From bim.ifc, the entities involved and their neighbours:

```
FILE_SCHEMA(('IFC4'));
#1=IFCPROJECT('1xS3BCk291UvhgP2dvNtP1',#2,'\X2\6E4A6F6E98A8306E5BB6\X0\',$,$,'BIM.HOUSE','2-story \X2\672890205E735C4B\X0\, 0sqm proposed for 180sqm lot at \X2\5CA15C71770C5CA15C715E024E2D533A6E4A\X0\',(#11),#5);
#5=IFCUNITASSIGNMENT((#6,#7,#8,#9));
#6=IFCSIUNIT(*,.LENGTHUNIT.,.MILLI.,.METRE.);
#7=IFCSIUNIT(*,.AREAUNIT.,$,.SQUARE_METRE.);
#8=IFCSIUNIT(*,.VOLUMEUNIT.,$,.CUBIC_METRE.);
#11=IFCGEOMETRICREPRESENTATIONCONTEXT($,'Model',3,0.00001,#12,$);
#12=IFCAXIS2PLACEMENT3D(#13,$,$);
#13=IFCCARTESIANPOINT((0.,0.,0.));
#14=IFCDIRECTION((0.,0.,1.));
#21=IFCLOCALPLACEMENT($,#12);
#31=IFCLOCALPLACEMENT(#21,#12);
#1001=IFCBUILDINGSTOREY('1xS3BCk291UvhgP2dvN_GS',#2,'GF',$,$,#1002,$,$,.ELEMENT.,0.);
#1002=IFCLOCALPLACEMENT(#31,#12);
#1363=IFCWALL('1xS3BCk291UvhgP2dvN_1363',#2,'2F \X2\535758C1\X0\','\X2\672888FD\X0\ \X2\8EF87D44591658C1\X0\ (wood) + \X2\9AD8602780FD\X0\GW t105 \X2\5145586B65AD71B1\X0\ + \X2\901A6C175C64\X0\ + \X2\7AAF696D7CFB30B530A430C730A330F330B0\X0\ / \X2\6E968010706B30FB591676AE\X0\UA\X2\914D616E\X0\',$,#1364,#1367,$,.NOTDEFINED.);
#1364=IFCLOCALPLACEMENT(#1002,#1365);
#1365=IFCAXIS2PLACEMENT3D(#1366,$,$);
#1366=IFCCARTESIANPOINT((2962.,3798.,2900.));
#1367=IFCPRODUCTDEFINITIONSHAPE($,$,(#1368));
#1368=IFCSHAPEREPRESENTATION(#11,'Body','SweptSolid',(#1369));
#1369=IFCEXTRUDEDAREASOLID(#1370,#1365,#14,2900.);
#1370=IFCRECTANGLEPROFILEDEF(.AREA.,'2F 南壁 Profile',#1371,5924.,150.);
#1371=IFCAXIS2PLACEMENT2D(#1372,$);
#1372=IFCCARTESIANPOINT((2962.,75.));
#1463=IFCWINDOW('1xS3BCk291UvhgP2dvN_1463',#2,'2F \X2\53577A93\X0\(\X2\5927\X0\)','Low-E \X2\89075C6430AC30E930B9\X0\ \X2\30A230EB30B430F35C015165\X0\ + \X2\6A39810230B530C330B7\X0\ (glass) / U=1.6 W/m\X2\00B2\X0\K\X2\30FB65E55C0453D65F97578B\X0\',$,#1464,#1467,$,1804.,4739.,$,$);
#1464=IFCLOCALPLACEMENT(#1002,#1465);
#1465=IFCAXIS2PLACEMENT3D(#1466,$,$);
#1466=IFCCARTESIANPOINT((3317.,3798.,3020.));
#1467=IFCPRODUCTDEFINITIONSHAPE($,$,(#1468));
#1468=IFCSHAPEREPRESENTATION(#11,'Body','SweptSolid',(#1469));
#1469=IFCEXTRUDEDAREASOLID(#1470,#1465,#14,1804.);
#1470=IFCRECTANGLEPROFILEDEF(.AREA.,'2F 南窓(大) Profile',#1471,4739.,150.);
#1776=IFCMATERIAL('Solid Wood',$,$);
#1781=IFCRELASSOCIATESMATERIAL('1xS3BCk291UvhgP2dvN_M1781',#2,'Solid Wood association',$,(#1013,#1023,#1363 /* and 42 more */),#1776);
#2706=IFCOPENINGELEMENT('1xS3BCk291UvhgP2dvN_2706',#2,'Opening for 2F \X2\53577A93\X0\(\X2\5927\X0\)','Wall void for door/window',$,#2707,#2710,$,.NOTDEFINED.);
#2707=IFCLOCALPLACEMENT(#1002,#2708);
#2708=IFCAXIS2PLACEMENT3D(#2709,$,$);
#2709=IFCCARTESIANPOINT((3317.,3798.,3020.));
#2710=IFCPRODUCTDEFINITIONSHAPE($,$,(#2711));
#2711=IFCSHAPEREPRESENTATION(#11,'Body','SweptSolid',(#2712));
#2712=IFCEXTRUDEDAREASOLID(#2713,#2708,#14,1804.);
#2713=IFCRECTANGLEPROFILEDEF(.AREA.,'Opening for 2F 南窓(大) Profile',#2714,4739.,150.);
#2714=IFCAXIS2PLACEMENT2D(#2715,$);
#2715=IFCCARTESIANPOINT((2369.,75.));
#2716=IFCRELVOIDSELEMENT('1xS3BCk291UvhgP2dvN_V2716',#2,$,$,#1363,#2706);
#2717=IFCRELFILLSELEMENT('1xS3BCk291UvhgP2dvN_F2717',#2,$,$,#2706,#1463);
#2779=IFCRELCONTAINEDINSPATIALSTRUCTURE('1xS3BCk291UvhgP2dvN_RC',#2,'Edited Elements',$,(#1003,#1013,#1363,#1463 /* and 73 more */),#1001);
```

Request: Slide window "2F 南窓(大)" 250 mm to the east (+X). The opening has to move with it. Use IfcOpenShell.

```python
import ifcopenshell
import ifcopenshell.api.geometry
import ifcopenshell.util.placement
import ifcopenshell.util.unit

model = ifcopenshell.open("bim.ifc")
unit_scale = ifcopenshell.util.unit.calculate_unit_scale(model)

window = model.by_guid("1xS3BCk291UvhgP2dvN_1463")
opening = window.FillsVoids[0].RelatingOpeningElement
wall = opening.VoidsElements[0].RelatingBuildingElement

wall_matrix = ifcopenshell.util.placement.get_local_placement(wall.ObjectPlacement)
shift = wall_matrix[:3, 0] * 0.25 / unit_scale
before = ifcopenshell.util.placement.get_local_placement(window.ObjectPlacement)[:3, 3].copy()

# The window is not placed relative to its opening, so move both.
for product in (opening, window):
    matrix = ifcopenshell.util.placement.get_local_placement(product.ObjectPlacement)
    matrix[:3, 3] += shift
    ifcopenshell.api.geometry.edit_object_placement(model, product=product, matrix=matrix, is_si=False)

after = ifcopenshell.util.placement.get_local_placement(window.ObjectPlacement)[:3, 3]
print("window moved by", (after - before).round(3) + 0.0)

model.write("bim_updated.ifc")
```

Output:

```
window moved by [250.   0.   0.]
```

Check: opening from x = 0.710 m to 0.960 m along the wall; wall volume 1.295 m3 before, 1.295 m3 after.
